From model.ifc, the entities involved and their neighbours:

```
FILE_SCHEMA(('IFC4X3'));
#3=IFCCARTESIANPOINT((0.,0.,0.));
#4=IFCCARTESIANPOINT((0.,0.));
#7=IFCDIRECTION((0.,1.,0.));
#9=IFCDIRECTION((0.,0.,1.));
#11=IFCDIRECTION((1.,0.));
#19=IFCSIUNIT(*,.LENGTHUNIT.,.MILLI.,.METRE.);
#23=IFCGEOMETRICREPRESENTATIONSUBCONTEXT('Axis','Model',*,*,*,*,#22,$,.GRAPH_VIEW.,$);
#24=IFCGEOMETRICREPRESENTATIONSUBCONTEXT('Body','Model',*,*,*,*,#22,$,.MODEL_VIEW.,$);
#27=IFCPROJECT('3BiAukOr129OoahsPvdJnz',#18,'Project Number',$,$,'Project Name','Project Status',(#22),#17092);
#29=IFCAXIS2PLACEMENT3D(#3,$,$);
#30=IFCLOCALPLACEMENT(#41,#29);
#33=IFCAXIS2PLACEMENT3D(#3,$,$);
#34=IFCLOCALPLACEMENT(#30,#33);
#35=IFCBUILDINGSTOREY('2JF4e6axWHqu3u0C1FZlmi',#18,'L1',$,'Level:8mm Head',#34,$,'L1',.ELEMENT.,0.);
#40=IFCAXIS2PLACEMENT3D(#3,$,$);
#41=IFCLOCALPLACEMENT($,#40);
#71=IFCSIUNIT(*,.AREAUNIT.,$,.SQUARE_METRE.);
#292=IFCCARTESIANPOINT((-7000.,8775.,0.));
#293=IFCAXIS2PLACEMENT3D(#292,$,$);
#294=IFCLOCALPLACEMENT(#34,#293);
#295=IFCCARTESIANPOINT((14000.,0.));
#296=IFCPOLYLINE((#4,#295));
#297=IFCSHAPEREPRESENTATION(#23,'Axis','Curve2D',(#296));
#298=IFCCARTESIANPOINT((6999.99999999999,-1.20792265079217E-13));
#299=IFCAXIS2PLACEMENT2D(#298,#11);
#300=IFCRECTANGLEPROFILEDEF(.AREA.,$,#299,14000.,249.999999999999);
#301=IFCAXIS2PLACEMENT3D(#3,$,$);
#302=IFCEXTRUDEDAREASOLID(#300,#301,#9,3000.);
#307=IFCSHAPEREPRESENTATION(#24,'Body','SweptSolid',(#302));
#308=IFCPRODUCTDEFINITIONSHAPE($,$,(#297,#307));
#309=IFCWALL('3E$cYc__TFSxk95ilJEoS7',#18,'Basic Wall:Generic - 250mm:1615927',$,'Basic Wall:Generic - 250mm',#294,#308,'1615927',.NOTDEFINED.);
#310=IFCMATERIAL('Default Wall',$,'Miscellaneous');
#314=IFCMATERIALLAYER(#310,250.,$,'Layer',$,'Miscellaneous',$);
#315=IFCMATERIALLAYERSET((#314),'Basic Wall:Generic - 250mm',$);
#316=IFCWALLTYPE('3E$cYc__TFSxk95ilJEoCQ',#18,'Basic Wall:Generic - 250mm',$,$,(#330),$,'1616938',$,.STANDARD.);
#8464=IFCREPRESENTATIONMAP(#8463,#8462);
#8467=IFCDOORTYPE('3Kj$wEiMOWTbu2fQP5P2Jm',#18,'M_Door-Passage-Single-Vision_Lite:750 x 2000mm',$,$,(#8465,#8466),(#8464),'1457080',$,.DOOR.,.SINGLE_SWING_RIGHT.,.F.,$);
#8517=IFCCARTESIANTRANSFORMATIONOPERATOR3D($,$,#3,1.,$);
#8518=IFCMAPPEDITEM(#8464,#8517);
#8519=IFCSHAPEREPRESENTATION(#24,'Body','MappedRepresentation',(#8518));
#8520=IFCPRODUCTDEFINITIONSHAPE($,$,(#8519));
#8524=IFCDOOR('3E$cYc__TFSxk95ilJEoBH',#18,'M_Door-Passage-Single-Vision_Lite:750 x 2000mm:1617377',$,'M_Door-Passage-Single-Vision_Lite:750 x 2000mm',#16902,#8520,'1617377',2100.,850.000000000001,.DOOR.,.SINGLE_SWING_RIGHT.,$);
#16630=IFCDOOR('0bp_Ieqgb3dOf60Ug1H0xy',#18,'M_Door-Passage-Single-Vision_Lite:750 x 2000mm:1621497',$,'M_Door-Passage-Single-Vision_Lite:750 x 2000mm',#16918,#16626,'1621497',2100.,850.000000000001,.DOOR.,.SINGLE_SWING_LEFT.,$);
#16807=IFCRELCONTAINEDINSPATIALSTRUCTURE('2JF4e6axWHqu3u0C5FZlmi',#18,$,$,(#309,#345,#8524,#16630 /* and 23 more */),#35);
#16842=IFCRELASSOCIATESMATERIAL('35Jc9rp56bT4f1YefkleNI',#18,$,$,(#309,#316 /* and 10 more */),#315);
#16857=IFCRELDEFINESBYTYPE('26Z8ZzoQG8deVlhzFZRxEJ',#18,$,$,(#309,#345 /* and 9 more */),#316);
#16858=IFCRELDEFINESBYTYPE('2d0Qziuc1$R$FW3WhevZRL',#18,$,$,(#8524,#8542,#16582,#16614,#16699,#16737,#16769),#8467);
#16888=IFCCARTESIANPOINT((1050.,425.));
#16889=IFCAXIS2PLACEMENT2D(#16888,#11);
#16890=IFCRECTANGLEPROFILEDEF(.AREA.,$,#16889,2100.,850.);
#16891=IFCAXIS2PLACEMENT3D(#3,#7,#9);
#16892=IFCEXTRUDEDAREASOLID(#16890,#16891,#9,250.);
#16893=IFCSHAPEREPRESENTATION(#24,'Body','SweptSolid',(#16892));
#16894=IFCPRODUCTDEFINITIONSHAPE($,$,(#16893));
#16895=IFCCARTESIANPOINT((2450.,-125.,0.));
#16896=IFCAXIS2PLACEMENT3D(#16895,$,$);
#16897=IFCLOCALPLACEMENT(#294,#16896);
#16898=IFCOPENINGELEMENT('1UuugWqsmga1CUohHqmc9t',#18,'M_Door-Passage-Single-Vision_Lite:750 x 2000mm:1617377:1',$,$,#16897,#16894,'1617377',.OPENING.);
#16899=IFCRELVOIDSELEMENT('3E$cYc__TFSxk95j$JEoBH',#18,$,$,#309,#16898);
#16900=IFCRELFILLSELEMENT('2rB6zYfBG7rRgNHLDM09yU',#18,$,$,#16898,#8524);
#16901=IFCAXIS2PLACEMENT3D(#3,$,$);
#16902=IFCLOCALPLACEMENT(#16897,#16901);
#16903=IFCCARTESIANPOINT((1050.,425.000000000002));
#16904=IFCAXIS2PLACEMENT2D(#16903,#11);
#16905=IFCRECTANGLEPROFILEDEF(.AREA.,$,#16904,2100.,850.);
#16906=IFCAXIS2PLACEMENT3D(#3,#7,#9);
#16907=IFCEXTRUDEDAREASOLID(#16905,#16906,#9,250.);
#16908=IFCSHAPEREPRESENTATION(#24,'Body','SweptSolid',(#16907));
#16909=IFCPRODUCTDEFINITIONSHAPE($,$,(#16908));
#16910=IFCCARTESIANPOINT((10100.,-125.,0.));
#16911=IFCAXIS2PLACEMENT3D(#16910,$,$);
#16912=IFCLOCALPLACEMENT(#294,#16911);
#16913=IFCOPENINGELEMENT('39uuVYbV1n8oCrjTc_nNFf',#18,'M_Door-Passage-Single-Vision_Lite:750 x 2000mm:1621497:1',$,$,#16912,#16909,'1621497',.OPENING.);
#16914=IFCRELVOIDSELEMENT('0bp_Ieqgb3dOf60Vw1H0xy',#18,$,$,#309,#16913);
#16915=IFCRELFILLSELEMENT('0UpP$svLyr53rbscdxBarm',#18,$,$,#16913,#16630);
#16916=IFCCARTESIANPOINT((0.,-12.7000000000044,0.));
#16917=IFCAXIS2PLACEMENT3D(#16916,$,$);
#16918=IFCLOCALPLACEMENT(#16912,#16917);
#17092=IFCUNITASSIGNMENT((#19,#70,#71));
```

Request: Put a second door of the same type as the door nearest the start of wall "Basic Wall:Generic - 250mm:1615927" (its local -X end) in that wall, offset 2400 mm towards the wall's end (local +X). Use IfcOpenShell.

```python
import ifcopenshell
import ifcopenshell.api.feature
import ifcopenshell.api.geometry
import ifcopenshell.api.root
import ifcopenshell.geom
import ifcopenshell.util.element
import ifcopenshell.util.placement
import ifcopenshell.util.shape
import ifcopenshell.util.unit

model = ifcopenshell.open("model.ifc")
unit_scale = ifcopenshell.util.unit.calculate_unit_scale(model)
settings = ifcopenshell.geom.settings()


def volume(element):
    """Net volume in cubic metres, openings subtracted."""
    shape = ifcopenshell.geom.create_shape(settings, element)
    return ifcopenshell.util.shape.get_volume(shape.geometry)


def reuse_history(source, copy):
    """copy_class also copies each property set's owner history, people and application; keep the originals."""
    for rel in copy.IsDefinedBy:
        if rel.is_a("IfcRelDefinesByProperties") and (history := rel.RelatingPropertyDefinition.OwnerHistory):
            rel.RelatingPropertyDefinition.OwnerHistory = source.OwnerHistory
            ifcopenshell.util.element.remove_deep2(model, history)


door = model.by_guid("3E$cYc__TFSxk95ilJEoBH")
opening = door.FillsVoids[0].RelatingOpeningElement
wall = opening.VoidsElements[0].RelatingBuildingElement
before = volume(wall)
shift = ifcopenshell.util.placement.get_local_placement(wall.ObjectPlacement)[:3, 0] * 2.4 / unit_scale

# copy_class copies the void relationship, type, container and properties, but no geometry.
new_opening = ifcopenshell.api.root.copy_class(model, product=opening)
new_opening.Representation = ifcopenshell.util.element.copy_deep(
    model, opening.Representation, exclude=["IfcGeometricRepresentationContext", "IfcRepresentationMap"]
)
new_opening.Name = "M_Door-Passage-Single-Vision_Lite:750 x 2000mm"
new_opening.Tag = None
new_door = ifcopenshell.api.root.copy_class(model, product=door)
new_door.Representation = ifcopenshell.util.element.copy_deep(
    model, door.Representation, exclude=["IfcGeometricRepresentationContext", "IfcRepresentationMap"]
)
new_door.Name = "M_Door-Passage-Single-Vision_Lite:750 x 2000mm"
new_door.Tag = None
reuse_history(door, new_door)
ifcopenshell.api.feature.add_filling(model, opening=new_opening, element=new_door)

for old, new in ((opening, new_opening), (door, new_door)):
    matrix = ifcopenshell.util.placement.get_local_placement(old.ObjectPlacement)
    matrix[:3, 3] += shift
    ifcopenshell.api.geometry.edit_object_placement(model, product=new, matrix=matrix, is_si=False)

after = volume(wall)

print(f"wall volume {before:.3f} -> {after:.3f} m3")

model.write("model_edited.ifc")
```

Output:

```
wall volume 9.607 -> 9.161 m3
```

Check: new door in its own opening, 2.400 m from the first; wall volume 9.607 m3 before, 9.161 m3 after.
